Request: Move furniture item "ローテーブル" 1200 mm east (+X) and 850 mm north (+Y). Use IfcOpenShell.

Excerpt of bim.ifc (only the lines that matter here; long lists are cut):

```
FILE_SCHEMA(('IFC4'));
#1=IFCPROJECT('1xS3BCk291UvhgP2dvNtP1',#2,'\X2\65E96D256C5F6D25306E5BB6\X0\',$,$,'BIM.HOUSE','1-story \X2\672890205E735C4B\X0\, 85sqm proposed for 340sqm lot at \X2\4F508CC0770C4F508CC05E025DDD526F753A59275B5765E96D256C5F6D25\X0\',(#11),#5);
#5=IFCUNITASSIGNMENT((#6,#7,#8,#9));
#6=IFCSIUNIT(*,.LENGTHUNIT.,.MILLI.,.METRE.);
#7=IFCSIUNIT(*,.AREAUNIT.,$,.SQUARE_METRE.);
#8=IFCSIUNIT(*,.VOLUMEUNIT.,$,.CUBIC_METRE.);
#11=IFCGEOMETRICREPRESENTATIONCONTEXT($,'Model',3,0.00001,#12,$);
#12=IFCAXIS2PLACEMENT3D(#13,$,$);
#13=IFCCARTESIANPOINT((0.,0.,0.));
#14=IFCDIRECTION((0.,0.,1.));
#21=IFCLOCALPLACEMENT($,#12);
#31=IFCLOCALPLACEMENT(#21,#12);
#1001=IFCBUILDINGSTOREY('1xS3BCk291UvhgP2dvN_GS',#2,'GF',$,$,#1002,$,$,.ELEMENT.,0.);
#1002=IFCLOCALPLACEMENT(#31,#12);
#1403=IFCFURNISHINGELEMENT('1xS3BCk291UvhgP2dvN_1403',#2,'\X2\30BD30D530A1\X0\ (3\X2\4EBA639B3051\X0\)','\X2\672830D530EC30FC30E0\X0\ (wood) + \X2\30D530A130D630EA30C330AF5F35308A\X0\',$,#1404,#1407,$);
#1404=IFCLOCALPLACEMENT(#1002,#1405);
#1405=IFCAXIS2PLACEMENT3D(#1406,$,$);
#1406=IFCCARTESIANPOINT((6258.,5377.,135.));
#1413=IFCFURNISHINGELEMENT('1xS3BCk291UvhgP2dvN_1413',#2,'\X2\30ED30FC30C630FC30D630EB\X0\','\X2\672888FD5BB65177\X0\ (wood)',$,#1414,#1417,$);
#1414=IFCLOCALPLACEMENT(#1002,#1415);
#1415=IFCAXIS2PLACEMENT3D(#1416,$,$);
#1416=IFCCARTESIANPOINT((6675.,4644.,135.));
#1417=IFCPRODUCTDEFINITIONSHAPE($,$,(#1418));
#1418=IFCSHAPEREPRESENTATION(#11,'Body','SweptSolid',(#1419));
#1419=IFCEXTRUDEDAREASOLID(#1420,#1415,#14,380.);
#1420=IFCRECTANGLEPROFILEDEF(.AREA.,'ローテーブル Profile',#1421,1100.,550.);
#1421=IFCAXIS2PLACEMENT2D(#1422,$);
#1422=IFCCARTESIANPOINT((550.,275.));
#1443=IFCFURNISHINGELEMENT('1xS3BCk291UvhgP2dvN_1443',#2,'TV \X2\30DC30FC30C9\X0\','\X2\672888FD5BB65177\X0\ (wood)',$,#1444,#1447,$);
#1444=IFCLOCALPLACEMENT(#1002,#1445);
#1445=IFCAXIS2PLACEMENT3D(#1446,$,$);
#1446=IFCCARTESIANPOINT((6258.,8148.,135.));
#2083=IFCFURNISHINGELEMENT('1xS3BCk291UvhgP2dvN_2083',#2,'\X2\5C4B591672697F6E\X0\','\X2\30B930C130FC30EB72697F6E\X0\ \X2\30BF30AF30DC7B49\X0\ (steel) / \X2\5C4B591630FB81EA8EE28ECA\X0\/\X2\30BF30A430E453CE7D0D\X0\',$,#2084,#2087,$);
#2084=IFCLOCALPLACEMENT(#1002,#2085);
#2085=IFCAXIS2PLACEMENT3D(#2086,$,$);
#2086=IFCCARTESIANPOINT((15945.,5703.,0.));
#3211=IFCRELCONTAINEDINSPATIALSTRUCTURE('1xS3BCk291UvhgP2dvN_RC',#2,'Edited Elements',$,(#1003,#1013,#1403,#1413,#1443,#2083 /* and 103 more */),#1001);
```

```python
import ifcopenshell
import ifcopenshell.api.geometry
import ifcopenshell.util.placement

model = ifcopenshell.open("bim.ifc")

item = model.by_guid("1xS3BCk291UvhgP2dvN_1413")
matrix = ifcopenshell.util.placement.get_local_placement(item.ObjectPlacement)
matrix[0, 3] += 1200.0
matrix[1, 3] += 850.0
ifcopenshell.api.geometry.edit_object_placement(model, product=item, matrix=matrix, is_si=False)

print(ifcopenshell.util.placement.get_local_placement(item.ObjectPlacement).round(3) + 0.0)

model.write("bim_v2.ifc")
```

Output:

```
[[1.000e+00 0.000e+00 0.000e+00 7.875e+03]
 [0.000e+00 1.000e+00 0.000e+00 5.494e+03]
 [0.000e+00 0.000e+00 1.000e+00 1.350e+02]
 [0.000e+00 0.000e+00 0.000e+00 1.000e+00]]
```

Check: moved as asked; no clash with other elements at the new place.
